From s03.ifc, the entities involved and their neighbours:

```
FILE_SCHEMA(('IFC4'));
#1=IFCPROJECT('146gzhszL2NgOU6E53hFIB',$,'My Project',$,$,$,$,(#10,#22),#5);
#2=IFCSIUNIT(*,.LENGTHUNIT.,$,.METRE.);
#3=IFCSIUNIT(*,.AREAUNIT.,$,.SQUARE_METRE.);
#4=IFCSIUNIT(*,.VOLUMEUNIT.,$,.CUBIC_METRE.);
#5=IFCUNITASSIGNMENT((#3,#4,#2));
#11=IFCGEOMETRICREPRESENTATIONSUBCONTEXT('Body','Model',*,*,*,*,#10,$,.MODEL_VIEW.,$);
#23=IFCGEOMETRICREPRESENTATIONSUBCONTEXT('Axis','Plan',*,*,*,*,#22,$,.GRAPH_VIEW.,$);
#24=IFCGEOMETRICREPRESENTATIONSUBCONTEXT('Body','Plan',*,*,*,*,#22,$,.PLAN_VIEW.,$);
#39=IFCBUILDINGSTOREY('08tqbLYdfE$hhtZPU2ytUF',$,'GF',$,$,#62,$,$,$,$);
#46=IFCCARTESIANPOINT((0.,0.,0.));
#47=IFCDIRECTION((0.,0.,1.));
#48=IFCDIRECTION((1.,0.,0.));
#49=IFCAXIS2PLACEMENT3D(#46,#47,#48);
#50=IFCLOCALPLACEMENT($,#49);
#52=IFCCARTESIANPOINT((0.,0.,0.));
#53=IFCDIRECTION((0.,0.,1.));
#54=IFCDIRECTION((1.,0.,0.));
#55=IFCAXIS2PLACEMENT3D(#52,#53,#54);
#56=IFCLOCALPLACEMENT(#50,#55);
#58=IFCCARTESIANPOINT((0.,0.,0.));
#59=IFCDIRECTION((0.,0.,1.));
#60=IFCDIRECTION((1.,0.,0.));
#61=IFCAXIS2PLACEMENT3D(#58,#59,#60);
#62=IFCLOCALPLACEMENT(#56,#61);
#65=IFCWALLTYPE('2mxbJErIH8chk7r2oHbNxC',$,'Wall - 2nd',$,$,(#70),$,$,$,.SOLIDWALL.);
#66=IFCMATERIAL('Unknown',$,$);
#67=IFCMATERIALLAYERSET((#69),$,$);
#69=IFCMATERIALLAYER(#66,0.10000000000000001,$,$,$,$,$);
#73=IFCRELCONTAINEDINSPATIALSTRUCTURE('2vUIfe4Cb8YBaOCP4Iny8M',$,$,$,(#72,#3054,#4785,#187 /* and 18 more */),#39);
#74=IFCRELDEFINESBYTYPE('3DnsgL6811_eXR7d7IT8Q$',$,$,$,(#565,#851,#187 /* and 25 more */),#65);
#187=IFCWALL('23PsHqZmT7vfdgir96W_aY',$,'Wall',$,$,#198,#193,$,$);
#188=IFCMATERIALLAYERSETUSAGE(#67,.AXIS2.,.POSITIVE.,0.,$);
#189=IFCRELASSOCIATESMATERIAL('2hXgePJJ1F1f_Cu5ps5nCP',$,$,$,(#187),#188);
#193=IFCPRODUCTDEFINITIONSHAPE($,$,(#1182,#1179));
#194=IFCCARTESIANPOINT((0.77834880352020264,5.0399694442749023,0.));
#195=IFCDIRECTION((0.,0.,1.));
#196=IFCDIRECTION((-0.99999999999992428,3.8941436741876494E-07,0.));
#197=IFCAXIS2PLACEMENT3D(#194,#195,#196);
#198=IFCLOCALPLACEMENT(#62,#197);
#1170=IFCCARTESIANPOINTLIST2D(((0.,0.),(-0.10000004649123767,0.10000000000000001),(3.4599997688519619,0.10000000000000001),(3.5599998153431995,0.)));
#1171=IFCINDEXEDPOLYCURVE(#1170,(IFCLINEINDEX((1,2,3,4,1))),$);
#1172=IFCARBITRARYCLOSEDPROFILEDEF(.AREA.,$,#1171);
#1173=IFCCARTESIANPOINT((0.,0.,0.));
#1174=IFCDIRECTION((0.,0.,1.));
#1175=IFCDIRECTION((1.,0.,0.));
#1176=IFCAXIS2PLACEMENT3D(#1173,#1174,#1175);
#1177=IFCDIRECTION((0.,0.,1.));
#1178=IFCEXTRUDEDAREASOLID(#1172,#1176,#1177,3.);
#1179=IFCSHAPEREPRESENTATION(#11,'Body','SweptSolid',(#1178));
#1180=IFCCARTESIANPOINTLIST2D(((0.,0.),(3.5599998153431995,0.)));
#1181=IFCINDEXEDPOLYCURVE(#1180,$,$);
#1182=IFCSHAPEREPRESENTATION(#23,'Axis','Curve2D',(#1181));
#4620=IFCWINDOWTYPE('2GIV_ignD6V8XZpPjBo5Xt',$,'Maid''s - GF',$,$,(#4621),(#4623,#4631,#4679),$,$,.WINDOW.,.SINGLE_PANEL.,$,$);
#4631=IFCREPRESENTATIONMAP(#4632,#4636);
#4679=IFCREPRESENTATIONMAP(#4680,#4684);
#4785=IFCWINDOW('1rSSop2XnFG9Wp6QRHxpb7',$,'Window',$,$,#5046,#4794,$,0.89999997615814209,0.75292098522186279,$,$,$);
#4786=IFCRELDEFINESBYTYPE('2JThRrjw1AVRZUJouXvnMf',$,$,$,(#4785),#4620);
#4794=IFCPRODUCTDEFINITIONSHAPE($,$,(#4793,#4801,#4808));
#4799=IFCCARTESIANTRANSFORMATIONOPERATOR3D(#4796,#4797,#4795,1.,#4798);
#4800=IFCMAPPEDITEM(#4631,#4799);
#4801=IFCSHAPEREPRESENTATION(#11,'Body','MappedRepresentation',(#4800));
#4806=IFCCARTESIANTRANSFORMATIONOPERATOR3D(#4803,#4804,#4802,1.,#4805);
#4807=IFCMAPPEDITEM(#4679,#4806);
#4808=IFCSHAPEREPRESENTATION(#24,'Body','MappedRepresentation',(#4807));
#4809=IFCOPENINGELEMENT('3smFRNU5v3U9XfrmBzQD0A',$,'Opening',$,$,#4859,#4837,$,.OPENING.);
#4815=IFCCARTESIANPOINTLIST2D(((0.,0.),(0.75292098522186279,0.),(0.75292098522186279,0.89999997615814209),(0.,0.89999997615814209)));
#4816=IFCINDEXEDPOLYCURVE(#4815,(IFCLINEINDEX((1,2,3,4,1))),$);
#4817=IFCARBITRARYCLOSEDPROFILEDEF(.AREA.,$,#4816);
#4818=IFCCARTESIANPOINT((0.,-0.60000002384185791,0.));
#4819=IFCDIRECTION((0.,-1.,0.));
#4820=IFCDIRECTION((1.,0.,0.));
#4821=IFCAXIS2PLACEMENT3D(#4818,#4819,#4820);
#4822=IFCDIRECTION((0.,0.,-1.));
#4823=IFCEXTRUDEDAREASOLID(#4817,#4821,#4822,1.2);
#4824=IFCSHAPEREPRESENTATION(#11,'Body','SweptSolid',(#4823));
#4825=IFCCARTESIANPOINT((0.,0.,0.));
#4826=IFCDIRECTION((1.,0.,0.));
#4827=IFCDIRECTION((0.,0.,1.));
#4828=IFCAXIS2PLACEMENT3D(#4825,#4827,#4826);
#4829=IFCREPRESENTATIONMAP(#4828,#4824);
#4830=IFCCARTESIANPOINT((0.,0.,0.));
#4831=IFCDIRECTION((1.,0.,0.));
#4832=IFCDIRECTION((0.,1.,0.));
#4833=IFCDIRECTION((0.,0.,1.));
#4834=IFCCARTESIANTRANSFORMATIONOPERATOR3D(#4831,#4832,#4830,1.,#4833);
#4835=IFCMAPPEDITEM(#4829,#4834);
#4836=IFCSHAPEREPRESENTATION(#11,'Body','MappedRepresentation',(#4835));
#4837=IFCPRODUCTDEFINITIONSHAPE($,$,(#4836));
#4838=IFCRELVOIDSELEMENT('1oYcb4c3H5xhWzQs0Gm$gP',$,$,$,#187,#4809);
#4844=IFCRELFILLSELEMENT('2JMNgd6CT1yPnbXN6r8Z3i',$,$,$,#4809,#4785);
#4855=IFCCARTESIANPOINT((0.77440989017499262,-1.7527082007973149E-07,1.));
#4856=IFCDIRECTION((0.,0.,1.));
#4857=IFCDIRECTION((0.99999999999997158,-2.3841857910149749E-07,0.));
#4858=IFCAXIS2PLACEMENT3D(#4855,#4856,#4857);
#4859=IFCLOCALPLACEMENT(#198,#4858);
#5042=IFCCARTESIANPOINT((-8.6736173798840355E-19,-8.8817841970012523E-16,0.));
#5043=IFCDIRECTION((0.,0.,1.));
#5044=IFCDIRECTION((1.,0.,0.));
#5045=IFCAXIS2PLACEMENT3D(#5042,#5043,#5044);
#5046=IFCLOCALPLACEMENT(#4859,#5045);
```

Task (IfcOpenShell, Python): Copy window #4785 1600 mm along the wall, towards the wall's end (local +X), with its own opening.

```python
import ifcopenshell
import ifcopenshell.api.feature
import ifcopenshell.api.geometry
import ifcopenshell.api.root
import ifcopenshell.geom
import ifcopenshell.util.element
import ifcopenshell.util.placement
import ifcopenshell.util.shape

model = ifcopenshell.open("s03.ifc")
settings = ifcopenshell.geom.settings()


def volume(element):
    """Net volume in cubic metres, openings subtracted."""
    shape = ifcopenshell.geom.create_shape(settings, element)
    return ifcopenshell.util.shape.get_volume(shape.geometry)


window = model.by_guid("1rSSop2XnFG9Wp6QRHxpb7")
opening = window.FillsVoids[0].RelatingOpeningElement
wall = opening.VoidsElements[0].RelatingBuildingElement
before = volume(wall)
shift = ifcopenshell.util.placement.get_local_placement(wall.ObjectPlacement)[:3, 0] * 1.6

# copy_class copies the void relationship, type, container and properties, but no geometry.
new_opening = ifcopenshell.api.root.copy_class(model, product=opening)
new_opening.Representation = ifcopenshell.util.element.copy_deep(
    model, opening.Representation, exclude=["IfcGeometricRepresentationContext", "IfcRepresentationMap"]
)
new_window = ifcopenshell.api.root.copy_class(model, product=window)
new_window.Representation = ifcopenshell.util.element.copy_deep(
    model, window.Representation, exclude=["IfcGeometricRepresentationContext", "IfcRepresentationMap"]
)
ifcopenshell.api.feature.add_filling(model, opening=new_opening, element=new_window)

for old, new in ((opening, new_opening), (window, new_window)):
    matrix = ifcopenshell.util.placement.get_local_placement(old.ObjectPlacement)
    matrix[:3, 3] += shift
    ifcopenshell.api.geometry.edit_object_placement(model, product=new, matrix=matrix, is_si=False)

after = volume(wall)

print(f"wall volume {before:.3f} -> {after:.3f} m3")

model.write("s03_updated.ifc")
```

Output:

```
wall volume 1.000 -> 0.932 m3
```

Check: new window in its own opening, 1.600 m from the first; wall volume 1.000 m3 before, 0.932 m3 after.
